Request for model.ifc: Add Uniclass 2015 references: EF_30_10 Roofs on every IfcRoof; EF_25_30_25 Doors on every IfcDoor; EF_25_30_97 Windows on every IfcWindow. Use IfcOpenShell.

First a look at what the model holds.

```python
import ifcopenshell

model = ifcopenshell.open("model.ifc")
print(model.schema)
print("classifications:", [c.Name for c in model.by_type("IfcClassification")])
for ifc_class in ("IfcDoor", "IfcRoof", "IfcStair", "IfcWall", "IfcWindow"):
    print(ifc_class, len(model.by_type(ifc_class)))
```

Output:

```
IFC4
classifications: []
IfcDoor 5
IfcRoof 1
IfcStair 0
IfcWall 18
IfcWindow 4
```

```python
import ifcopenshell
import ifcopenshell.api.classification

model = ifcopenshell.open("model.ifc")

system = ifcopenshell.api.classification.add_classification(model, classification="Uniclass 2015")

codes = {
    "IfcRoof": ("EF_30_10", "Roofs"),
    "IfcDoor": ("EF_25_30_25", "Doors"),
    "IfcWindow": ("EF_25_30_97", "Windows"),
}
for ifc_class, (code, name) in codes.items():
    products = model.by_type(ifc_class)
    ifcopenshell.api.classification.add_reference(
        model, products=products, classification=system, identification=code, name=name
    )
    print(code, len(products))

model.write("model_edited.ifc")
```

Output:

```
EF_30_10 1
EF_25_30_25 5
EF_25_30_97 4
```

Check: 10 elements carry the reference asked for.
